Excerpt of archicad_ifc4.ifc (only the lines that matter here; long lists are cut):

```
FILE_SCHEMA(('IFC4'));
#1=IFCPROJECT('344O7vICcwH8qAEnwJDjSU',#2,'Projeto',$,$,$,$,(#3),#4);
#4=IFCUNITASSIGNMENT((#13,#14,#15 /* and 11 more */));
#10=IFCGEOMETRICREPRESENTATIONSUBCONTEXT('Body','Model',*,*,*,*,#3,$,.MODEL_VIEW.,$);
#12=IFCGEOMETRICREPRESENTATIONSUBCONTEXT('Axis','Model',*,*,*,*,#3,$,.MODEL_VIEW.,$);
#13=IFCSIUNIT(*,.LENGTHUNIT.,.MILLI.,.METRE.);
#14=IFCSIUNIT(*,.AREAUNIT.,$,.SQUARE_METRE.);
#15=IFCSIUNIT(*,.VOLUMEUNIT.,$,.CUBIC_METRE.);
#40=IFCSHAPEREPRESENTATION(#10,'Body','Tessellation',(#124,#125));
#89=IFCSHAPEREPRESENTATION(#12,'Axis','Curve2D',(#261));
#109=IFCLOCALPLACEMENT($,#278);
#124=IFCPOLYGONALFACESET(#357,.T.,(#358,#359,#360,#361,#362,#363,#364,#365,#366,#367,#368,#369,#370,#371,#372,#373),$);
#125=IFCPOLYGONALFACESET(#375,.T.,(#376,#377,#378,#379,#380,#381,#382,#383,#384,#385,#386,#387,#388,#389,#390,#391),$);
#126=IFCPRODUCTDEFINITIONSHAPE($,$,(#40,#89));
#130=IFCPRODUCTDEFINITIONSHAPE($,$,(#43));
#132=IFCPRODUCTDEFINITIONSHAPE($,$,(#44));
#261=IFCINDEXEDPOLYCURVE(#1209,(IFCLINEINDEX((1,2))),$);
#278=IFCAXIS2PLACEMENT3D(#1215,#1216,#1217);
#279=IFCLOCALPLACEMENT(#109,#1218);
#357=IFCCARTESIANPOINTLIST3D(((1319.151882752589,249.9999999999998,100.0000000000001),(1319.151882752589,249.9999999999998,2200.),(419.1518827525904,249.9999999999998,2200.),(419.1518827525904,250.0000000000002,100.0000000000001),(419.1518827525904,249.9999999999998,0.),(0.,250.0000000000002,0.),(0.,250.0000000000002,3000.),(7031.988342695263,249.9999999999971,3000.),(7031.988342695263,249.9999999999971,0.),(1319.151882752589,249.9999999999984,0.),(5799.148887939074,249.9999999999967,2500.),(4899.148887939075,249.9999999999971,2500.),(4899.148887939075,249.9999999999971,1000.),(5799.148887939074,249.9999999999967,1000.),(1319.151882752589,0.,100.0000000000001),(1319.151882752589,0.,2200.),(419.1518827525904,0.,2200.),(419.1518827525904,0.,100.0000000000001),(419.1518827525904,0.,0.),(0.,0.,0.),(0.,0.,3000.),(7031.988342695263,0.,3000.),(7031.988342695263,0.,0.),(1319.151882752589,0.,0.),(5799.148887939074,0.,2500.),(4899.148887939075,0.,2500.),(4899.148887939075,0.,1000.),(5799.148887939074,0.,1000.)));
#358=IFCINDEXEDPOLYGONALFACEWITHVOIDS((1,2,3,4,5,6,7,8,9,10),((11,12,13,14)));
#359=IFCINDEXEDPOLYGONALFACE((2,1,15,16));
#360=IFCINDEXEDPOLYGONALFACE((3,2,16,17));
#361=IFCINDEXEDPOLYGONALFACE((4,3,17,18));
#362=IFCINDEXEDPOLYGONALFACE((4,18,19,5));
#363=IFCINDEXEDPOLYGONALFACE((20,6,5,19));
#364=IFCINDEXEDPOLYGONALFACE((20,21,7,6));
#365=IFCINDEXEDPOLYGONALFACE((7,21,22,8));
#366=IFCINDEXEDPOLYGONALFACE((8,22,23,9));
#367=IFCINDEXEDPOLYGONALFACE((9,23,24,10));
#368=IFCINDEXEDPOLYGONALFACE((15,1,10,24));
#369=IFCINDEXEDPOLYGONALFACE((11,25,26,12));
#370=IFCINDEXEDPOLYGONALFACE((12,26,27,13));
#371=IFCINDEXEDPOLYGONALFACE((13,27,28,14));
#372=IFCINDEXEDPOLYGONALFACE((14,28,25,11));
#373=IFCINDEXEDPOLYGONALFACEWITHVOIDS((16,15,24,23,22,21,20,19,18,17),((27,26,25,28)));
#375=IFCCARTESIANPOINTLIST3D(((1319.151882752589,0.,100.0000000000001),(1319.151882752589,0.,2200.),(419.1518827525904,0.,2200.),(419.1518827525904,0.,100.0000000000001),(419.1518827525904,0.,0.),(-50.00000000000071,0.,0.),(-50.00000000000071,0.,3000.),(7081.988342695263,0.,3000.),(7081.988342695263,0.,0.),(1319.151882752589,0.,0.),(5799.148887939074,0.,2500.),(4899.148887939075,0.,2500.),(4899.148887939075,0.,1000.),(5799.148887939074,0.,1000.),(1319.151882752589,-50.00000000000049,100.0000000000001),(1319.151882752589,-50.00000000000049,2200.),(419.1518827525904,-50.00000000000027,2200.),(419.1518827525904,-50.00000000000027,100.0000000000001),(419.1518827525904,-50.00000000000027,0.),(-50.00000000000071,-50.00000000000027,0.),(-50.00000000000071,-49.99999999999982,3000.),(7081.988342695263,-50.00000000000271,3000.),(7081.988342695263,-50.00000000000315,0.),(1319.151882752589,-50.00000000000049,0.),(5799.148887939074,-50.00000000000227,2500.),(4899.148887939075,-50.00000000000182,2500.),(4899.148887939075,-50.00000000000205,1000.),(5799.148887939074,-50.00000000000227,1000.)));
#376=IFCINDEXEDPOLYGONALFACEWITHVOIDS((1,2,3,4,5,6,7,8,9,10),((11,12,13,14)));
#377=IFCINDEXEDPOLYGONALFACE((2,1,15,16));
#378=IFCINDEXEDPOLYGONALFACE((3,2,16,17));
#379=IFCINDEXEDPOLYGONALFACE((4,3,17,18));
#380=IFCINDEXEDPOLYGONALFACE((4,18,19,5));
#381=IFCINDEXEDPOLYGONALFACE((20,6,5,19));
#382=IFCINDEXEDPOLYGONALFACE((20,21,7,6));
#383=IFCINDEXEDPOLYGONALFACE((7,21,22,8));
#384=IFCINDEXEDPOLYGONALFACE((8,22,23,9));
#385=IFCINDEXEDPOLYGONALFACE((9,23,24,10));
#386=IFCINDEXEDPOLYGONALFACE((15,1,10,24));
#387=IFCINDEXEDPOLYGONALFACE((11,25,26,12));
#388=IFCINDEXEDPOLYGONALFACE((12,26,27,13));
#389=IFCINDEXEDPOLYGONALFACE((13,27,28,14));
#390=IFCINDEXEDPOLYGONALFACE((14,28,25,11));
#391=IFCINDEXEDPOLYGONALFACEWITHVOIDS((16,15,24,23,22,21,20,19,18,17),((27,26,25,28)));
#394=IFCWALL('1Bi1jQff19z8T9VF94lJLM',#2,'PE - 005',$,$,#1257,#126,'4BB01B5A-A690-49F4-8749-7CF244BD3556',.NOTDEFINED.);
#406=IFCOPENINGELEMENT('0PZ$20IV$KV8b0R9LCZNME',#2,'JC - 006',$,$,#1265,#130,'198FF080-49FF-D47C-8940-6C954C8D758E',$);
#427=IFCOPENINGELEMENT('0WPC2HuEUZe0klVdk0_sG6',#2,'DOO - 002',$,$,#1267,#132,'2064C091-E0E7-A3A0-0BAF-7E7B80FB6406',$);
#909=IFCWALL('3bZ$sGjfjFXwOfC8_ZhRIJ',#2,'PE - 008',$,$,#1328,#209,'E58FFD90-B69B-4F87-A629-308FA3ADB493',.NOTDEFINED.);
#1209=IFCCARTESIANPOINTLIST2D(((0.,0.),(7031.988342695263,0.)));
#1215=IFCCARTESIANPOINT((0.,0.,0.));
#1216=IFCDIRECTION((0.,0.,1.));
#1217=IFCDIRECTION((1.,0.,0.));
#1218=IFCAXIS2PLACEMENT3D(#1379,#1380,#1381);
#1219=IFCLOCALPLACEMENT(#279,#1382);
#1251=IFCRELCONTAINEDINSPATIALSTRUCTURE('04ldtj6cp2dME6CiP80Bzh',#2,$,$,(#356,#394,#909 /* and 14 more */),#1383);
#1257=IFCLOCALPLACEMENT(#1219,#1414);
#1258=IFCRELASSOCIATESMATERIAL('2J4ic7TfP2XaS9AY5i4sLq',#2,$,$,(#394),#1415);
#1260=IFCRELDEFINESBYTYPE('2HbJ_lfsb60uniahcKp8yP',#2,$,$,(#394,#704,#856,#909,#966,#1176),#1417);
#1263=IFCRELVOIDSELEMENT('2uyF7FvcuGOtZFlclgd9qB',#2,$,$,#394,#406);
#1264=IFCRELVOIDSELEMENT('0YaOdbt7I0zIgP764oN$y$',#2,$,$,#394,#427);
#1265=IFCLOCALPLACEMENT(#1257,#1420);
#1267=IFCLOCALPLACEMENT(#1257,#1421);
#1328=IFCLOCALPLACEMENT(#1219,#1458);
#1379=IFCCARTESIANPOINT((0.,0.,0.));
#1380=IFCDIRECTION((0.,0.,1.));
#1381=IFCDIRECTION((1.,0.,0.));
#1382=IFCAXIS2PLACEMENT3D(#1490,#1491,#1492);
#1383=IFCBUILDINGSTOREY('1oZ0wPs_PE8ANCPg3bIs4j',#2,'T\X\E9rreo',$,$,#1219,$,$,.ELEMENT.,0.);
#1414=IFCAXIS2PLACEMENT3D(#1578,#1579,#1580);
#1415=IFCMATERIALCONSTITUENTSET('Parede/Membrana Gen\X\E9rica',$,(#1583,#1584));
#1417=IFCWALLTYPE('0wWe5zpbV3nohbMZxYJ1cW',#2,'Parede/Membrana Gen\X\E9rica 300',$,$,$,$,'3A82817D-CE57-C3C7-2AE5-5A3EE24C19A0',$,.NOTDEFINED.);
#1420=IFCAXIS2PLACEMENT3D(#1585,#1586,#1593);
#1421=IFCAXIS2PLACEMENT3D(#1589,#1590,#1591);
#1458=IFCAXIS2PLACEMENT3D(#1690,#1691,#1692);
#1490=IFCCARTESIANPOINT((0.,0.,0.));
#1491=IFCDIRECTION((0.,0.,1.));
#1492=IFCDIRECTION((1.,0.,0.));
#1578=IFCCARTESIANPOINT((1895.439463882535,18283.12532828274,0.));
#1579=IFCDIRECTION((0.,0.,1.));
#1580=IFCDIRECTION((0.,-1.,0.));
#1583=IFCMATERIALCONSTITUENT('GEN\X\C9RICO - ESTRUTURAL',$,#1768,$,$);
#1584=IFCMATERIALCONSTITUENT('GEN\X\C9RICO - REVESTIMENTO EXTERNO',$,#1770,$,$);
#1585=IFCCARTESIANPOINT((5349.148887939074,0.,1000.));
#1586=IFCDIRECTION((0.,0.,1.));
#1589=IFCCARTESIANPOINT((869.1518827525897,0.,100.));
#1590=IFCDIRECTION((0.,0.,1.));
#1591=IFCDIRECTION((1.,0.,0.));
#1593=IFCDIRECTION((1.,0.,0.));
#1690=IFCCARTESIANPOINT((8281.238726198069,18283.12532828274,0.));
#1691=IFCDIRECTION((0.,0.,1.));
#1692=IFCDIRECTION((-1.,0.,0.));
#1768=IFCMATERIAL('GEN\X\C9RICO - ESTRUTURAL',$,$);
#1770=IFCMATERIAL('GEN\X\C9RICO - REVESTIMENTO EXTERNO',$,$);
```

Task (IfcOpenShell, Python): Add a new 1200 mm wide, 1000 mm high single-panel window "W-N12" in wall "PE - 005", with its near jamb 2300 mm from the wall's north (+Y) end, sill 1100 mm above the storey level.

```python
import numpy as np
import ifcopenshell
import ifcopenshell.api.feature
import ifcopenshell.api.geometry
import ifcopenshell.api.root
import ifcopenshell.api.spatial
import ifcopenshell.geom
import ifcopenshell.util.element
import ifcopenshell.util.placement
import ifcopenshell.util.representation
import ifcopenshell.util.shape
import ifcopenshell.util.unit

model = ifcopenshell.open("archicad_ifc4.ifc")
unit_scale = ifcopenshell.util.unit.calculate_unit_scale(model)
settings = ifcopenshell.geom.settings()


def volume(element):
    """Net volume in cubic metres, openings subtracted."""
    shape = ifcopenshell.geom.create_shape(settings, element)
    return ifcopenshell.util.shape.get_volume(shape.geometry)


wall = model.by_guid("1Bi1jQff19z8T9VF94lJLM")
storey = ifcopenshell.util.element.get_container(wall, ifc_class="IfcBuildingStorey")
context = ifcopenshell.util.representation.get_context(model, "Model", "Body", "MODEL_VIEW")
before = volume(wall)

width, height, from_end, sill = 1.2, 1, 2.3, 1.1  # metres

# The wall runs along its own X axis, and the end named is its -X end.
wall_shape = ifcopenshell.geom.create_shape(settings, wall)
x, y, z = ifcopenshell.util.shape.get_vertices(wall_shape.geometry).T
start = x.min() + from_end
face, thickness = float(y.min()), float(y.max() - y.min())
wall_matrix = ifcopenshell.util.placement.get_local_placement(wall.ObjectPlacement)
level = ifcopenshell.util.placement.get_local_placement(storey.ObjectPlacement)[2, 3]


def in_wall(x, y):
    """Placement at x, y metres in the wall's axes, at sill height."""
    matrix = wall_matrix.copy()
    matrix[:, 3] = wall_matrix @ np.array([x / unit_scale, y / unit_scale, 0.0, 1.0])
    matrix[2, 3] = level + sill / unit_scale
    return matrix


# Opening: a box that overshoots both wall faces by 50 mm.
opening = ifcopenshell.api.root.create_entity(model, ifc_class="IfcOpeningElement", predefined_type="OPENING")
box = ifcopenshell.api.geometry.add_wall_representation(
    model, context=context, length=width, height=height, thickness=thickness + 0.1
)
ifcopenshell.api.geometry.assign_representation(model, product=opening, representation=box)
ifcopenshell.api.geometry.edit_object_placement(model, product=opening, matrix=in_wall(start, face - 0.05), is_si=False)
ifcopenshell.api.feature.add_feature(model, feature=opening, element=wall)

window = ifcopenshell.api.root.create_entity(model, ifc_class="IfcWindow", name="W-N12", predefined_type="WINDOW")
window.OverallWidth, window.OverallHeight = width / unit_scale, height / unit_scale
window.PartitioningType = "SINGLE_PANEL"
body = ifcopenshell.api.geometry.add_window_representation(
    model,
    context=context,
    overall_width=window.OverallWidth,
    overall_height=window.OverallHeight,
    partition_type="SINGLE_PANEL",
)
ifcopenshell.api.geometry.assign_representation(model, product=window, representation=body)
ifcopenshell.api.spatial.assign_container(model, products=[window], relating_structure=storey)
ifcopenshell.api.feature.add_filling(model, opening=opening, element=window)

# Centre the window in the wall's thickness.
ifcopenshell.api.geometry.edit_object_placement(model, product=window, matrix=in_wall(start, face), is_si=False)
window_shape = ifcopenshell.geom.create_shape(settings, window)
depth = ifcopenshell.util.shape.get_vertices(window_shape.geometry)[:, 1]
offset = face + thickness / 2 - (depth.min() + depth.max()) / 2
ifcopenshell.api.geometry.edit_object_placement(model, product=window, matrix=in_wall(start, offset), is_si=False)

after = volume(wall)

print(f"wall volume {before:.3f} -> {after:.3f} m3")

model.write("archicad_ifc4_edited.ifc")
```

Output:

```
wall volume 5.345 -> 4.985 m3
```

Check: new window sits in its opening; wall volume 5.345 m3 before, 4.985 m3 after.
